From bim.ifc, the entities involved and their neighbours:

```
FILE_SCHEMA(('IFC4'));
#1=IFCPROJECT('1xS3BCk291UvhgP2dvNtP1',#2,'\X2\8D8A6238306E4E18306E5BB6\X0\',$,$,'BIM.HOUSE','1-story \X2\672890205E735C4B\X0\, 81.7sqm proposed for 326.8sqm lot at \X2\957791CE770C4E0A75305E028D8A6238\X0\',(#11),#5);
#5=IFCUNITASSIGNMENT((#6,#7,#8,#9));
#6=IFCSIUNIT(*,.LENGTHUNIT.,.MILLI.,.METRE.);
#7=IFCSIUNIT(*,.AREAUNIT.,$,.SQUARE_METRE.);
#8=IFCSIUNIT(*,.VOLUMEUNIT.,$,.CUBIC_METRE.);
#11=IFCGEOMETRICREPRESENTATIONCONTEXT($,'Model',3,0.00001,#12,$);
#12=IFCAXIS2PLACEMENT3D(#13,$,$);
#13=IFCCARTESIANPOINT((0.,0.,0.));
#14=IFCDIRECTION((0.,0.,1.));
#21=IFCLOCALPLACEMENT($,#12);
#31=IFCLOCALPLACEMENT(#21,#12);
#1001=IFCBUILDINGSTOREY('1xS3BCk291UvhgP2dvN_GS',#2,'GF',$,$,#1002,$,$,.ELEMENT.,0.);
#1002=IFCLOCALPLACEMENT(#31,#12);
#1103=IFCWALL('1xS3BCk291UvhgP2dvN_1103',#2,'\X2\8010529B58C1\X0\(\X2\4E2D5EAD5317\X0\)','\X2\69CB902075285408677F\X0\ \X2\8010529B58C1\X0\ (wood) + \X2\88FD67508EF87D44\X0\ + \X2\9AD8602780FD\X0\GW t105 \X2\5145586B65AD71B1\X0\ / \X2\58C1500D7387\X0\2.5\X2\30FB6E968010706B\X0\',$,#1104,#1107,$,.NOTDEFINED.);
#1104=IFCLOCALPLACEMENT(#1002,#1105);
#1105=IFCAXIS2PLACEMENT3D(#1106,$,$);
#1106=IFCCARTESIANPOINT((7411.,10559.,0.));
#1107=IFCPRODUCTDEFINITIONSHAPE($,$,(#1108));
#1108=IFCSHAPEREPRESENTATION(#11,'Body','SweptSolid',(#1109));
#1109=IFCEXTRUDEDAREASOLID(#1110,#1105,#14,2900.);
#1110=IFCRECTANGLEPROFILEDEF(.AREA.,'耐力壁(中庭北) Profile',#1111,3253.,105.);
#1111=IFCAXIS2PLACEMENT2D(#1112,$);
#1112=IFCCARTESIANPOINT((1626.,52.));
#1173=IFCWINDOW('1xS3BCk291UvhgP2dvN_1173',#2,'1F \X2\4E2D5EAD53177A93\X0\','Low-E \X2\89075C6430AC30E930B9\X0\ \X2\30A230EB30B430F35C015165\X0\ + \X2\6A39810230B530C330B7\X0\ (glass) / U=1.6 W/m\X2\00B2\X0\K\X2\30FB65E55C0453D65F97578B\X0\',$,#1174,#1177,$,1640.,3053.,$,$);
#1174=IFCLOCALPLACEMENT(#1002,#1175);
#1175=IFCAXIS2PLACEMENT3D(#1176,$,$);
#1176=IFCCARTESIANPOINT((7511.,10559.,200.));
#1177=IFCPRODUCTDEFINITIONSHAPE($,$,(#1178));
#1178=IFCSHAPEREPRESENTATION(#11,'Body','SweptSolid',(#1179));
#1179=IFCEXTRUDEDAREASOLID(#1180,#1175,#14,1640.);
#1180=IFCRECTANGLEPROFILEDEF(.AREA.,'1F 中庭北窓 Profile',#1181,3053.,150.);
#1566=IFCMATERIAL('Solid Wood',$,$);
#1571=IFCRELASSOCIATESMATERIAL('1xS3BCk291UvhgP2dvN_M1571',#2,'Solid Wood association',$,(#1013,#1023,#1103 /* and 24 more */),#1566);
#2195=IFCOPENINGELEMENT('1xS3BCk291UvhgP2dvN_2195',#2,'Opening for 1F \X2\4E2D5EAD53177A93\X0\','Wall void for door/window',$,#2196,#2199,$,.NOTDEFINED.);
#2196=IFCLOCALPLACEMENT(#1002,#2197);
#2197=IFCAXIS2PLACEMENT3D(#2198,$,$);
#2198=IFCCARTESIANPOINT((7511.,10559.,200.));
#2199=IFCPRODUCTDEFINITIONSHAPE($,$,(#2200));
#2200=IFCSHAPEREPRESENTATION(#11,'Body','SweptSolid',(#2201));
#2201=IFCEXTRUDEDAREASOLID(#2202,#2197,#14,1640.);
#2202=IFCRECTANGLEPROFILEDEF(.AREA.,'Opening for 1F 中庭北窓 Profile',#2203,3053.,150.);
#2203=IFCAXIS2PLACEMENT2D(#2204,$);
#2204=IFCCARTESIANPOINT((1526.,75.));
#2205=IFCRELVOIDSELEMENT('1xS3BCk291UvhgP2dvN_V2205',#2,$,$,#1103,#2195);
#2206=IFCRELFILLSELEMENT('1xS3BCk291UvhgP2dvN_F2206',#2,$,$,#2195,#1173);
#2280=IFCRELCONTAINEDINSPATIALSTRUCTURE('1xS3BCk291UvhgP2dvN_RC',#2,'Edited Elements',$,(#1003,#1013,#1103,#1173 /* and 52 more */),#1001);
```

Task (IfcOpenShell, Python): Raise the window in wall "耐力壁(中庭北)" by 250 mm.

```python
import numpy as np
import ifcopenshell
import ifcopenshell.api.geometry
import ifcopenshell.util.placement
import ifcopenshell.util.unit

model = ifcopenshell.open("bim.ifc")
unit_scale = ifcopenshell.util.unit.calculate_unit_scale(model)

window = model.by_guid("1xS3BCk291UvhgP2dvN_1173")
opening = window.FillsVoids[0].RelatingOpeningElement
dz = 250.0

shift = np.array([0.0, 0.0, dz])
# The window is not placed relative to its opening, so move both.
for product in (opening, window):
    matrix = ifcopenshell.util.placement.get_local_placement(product.ObjectPlacement)
    matrix[:3, 3] += shift
    ifcopenshell.api.geometry.edit_object_placement(model, product=product, matrix=matrix, is_si=False)

print(f"moved by {dz * unit_scale:+.3f} m")

model.write("bim_v2.ifc")
```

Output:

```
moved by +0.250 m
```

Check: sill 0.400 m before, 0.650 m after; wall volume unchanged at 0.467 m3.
